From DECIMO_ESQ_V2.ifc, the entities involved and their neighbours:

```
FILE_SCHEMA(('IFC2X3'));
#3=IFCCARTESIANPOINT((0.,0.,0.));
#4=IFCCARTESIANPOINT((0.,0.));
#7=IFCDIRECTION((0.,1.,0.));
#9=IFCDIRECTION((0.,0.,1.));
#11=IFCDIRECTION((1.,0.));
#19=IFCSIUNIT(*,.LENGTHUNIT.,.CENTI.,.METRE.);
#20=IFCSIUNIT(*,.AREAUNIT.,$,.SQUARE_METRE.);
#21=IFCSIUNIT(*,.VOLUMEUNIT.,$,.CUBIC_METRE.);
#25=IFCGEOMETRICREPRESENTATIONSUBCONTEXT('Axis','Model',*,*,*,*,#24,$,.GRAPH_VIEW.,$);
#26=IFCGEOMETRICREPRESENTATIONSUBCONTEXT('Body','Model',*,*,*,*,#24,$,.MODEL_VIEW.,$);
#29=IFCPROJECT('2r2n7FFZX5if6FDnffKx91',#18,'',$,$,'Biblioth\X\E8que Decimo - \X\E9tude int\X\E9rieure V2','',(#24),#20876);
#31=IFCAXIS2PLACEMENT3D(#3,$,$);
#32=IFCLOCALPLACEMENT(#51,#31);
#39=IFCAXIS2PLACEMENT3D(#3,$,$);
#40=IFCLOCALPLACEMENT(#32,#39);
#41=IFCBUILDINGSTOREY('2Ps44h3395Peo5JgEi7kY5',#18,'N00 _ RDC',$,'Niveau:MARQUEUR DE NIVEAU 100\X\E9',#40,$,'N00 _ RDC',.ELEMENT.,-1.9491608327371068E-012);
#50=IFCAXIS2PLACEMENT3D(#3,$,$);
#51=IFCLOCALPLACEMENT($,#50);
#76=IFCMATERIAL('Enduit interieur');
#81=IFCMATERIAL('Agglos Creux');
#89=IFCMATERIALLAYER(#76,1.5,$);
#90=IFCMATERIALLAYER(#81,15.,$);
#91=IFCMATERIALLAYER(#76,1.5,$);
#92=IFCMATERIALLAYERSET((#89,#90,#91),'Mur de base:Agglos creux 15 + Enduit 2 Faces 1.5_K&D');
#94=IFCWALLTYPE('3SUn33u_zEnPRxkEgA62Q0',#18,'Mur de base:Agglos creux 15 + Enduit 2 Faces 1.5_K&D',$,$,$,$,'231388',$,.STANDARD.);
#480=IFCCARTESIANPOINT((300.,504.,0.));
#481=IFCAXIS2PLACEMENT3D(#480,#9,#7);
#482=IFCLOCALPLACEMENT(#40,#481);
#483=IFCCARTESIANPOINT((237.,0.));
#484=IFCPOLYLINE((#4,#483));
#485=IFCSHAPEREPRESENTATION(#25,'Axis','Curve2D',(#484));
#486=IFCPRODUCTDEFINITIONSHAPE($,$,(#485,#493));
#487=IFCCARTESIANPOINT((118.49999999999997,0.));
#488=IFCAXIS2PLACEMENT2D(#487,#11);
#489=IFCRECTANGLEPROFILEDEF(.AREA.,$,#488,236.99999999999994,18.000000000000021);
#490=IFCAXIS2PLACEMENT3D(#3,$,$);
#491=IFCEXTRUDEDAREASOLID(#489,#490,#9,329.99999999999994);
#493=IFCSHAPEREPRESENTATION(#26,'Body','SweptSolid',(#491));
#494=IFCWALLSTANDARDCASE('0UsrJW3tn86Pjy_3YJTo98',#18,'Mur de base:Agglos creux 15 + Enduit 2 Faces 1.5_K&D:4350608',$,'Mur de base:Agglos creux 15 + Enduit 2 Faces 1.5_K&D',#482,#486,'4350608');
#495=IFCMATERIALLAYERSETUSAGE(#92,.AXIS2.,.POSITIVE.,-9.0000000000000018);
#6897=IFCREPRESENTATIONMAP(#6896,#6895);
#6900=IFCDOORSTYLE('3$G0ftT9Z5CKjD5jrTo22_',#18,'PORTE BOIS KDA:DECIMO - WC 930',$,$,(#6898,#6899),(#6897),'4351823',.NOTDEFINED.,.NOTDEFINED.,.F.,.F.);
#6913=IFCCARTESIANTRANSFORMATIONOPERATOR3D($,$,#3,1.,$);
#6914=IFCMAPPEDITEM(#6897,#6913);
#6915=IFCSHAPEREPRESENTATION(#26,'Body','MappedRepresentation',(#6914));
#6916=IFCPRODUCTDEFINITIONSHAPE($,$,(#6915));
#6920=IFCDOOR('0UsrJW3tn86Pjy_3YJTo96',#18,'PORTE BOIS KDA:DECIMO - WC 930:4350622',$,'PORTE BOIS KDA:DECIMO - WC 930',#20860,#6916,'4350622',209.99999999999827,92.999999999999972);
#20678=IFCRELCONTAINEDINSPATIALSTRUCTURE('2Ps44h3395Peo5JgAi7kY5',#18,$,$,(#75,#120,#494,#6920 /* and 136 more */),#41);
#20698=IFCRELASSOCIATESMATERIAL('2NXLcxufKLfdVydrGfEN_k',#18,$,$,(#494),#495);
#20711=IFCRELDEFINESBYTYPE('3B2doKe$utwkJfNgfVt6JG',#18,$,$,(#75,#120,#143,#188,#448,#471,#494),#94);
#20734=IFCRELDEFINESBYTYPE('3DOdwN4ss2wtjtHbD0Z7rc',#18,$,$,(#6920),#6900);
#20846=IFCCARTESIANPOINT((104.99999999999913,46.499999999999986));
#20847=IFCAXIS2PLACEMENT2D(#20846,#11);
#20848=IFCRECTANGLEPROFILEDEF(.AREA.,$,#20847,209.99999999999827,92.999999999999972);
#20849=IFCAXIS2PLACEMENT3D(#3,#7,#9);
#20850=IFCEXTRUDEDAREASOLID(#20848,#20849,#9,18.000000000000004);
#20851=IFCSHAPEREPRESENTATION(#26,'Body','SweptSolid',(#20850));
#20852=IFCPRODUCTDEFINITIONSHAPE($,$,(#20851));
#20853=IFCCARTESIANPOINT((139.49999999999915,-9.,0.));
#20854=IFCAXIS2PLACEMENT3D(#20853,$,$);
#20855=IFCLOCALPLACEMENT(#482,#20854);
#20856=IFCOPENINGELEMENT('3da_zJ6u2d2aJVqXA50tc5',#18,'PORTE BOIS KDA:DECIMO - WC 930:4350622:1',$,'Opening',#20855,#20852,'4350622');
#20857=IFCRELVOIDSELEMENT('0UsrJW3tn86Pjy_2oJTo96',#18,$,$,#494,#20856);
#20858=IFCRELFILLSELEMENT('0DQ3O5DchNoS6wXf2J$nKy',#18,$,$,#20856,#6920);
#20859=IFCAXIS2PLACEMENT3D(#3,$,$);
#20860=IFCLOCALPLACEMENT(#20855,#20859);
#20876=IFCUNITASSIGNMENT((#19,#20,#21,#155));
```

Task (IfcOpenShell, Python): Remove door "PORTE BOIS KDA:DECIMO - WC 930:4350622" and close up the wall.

```python
import ifcopenshell
import ifcopenshell.api.feature
import ifcopenshell.api.root
import ifcopenshell.geom
import ifcopenshell.util.shape

model = ifcopenshell.open("DECIMO_ESQ_V2.ifc")
settings = ifcopenshell.geom.settings()


def volume(element):
    """Net volume in cubic metres, openings subtracted."""
    shape = ifcopenshell.geom.create_shape(settings, element)
    return ifcopenshell.util.shape.get_volume(shape.geometry)


door = model.by_id(6920)
opening = door.FillsVoids[0].RelatingOpeningElement
wall = opening.VoidsElements[0].RelatingBuildingElement
before = volume(wall)

ifcopenshell.api.root.remove_product(model, product=door)
ifcopenshell.api.feature.remove_feature(model, feature=opening)

after = volume(wall)

print(f"wall volume {before:.3f} -> {after:.3f} m3")

model.write("DECIMO_ESQ_V2_edited.ifc")
```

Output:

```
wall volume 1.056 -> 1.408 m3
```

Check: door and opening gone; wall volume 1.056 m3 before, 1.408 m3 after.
